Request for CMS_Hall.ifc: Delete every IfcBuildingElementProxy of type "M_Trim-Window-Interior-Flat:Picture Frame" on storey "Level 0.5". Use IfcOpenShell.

First a look at what the model holds.

```python
import ifcopenshell
import ifcopenshell.util.element

model = ifcopenshell.open("CMS_Hall.ifc")
print(model.schema)
storey = next(s for s in model.by_type("IfcBuildingStorey") if s.Name == "Level 0.5")
proxies = [e for e in ifcopenshell.util.element.get_decomposition(storey) if e.is_a("IfcBuildingElementProxy")]
seen = {}
for e in proxies:
    element_type = ifcopenshell.util.element.get_type(e)
    name = element_type.Name if element_type not in (None, e) else None
    seen[name] = seen.get(name, 0) + 1
for name, count in sorted(seen.items(), key=str):
    print(count, "x", name)
```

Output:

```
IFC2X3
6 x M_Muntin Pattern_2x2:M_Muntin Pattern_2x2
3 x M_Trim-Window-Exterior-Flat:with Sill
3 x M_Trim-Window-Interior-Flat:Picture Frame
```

```python
import ifcopenshell
import ifcopenshell.api.root
import ifcopenshell.util.element

model = ifcopenshell.open("CMS_Hall.ifc")

storey = next(s for s in model.by_type("IfcBuildingStorey") if s.Name == "Level 0.5")
proxies = [e for e in ifcopenshell.util.element.get_decomposition(storey) if e.is_a("IfcBuildingElementProxy")]
targets = [e for e in proxies if (t := ifcopenshell.util.element.get_type(e)) not in (None, e) and t.Name == "M_Trim-Window-Interior-Flat:Picture Frame"]

for e in targets:
    ifcopenshell.api.root.remove_product(model, product=e)
print(len(targets), "removed")

model.write("CMS_Hall_rev.ifc")
```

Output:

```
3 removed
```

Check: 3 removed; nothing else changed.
